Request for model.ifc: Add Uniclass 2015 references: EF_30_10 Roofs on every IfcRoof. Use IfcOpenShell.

First a look at what the model holds.

```python
import ifcopenshell

model = ifcopenshell.open("model.ifc")
print(model.schema)
print("classifications:", [c.Name for c in model.by_type("IfcClassification")])
for ifc_class in ("IfcDoor", "IfcRoof", "IfcStair", "IfcWall", "IfcWindow"):
    print(ifc_class, len(model.by_type(ifc_class)))
```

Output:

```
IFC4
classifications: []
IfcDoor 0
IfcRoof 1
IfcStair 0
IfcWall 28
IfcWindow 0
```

```python
import ifcopenshell
import ifcopenshell.api.classification

model = ifcopenshell.open("model.ifc")

system = ifcopenshell.api.classification.add_classification(model, classification="Uniclass 2015")

codes = {
    "IfcRoof": ("EF_30_10", "Roofs"),
}
for ifc_class, (code, name) in codes.items():
    products = model.by_type(ifc_class)
    ifcopenshell.api.classification.add_reference(
        model, products=products, classification=system, identification=code, name=name
    )
    print(code, len(products))

model.write("model_edited.ifc")
```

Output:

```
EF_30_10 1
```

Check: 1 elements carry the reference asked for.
